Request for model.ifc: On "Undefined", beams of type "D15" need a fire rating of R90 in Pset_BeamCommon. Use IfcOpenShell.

First a look at what the model holds.

```python
import ifcopenshell
import ifcopenshell.util.element

model = ifcopenshell.open("model.ifc")
print(model.schema)
storey = next(s for s in model.by_type("IfcBuildingStorey") if s.Name == "Undefined")
beams = [e for e in ifcopenshell.util.element.get_decomposition(storey) if e.is_a("IfcBeam")]
seen = {}
for e in beams:
    element_type = ifcopenshell.util.element.get_type(e)
    key = (element_type.Name if element_type != e and element_type else None, ifcopenshell.util.element.get_pset(e, "Pset_BeamCommon", "FireRating"))
    seen[key] = seen.get(key, 0) + 1
for (name, value), count in sorted(seen.items(), key=str):
    print(count, "x", name, "|", value)
```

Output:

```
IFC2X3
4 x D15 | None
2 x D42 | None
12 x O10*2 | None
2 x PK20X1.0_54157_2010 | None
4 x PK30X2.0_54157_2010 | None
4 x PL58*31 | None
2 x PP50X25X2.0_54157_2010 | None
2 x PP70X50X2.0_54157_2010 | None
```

```python
import ifcopenshell
import ifcopenshell.api.pset
import ifcopenshell.util.element

model = ifcopenshell.open("model.ifc")

storey = next(s for s in model.by_type("IfcBuildingStorey") if s.Name == "Undefined")
beams = [e for e in ifcopenshell.util.element.get_decomposition(storey) if e.is_a("IfcBeam")]

count = 0
for e in beams:
    element_type = ifcopenshell.util.element.get_type(e)
    if element_type in (None, e) or element_type.Name != "D15":
        continue
    found = ifcopenshell.util.element.get_pset(e, "Pset_BeamCommon", should_inherit=False)
    if found:
        pset = model.by_id(found["id"])
        if len(ifcopenshell.util.element.get_elements_by_pset(pset)) > 1:
            pset = ifcopenshell.api.pset.unshare_pset(model, products=[e], pset=pset)[0]
    else:
        pset = ifcopenshell.api.pset.add_pset(model, product=e, name="Pset_BeamCommon")
    ifcopenshell.api.pset.edit_pset(model, pset=pset, properties={"FireRating": "R90"})
    count += 1

print(count, "beams updated")

model.write("model-out.ifc")
```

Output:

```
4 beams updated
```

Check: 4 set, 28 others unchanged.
